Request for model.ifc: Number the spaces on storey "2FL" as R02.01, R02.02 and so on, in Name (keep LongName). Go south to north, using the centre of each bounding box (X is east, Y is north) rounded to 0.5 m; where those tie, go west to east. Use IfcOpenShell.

First a look at what the model holds.

```python
import ifcopenshell
import ifcopenshell.util.element
import ifcopenshell.util.placement

model = ifcopenshell.open("model.ifc")
print(model.schema)
storey = next(s for s in model.by_type("IfcBuildingStorey") if s.Name == "2FL")
spaces = [e for e in ifcopenshell.util.element.get_decomposition(storey) if e.is_a("IfcSpace")]
for e in sorted(spaces, key=lambda e: e.id()):
    origin = ifcopenshell.util.placement.get_local_placement(e.ObjectPlacement)[:3, 3]
    print(e.id(), e.Name, e.LongName, origin.round(2) + 0.0, sep=" | ")
```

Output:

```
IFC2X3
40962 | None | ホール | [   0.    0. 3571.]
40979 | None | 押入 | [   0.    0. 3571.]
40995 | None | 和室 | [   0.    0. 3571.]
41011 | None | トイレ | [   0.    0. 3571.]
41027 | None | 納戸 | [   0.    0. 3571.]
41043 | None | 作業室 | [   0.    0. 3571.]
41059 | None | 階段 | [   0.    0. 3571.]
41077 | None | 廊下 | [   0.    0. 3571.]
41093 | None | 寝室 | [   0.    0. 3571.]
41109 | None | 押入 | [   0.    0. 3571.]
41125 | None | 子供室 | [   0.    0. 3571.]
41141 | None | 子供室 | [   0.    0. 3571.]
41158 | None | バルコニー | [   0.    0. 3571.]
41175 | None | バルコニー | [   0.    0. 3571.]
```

```python
import ifcopenshell
import ifcopenshell.geom
import ifcopenshell.util.element
import ifcopenshell.util.shape

model = ifcopenshell.open("model.ifc")
settings = ifcopenshell.geom.settings()
settings.set("use-world-coords", True)


def centre(element):
    shape = ifcopenshell.geom.create_shape(settings, element)
    return ifcopenshell.util.shape.get_bbox_centroid(shape.geometry)


storey = next(s for s in model.by_type("IfcBuildingStorey") if s.Name == "2FL")
spaces = [e for e in ifcopenshell.util.element.get_decomposition(storey) if e.is_a("IfcSpace")]

# Insertion points can sit at a corner or the storey origin, so sort by the geometry (in metres).
centres = {e: centre(e) for e in spaces}
spaces.sort(key=lambda e: (round(centres[e][1] / 0.5), centres[e][0]))

for i, e in enumerate(spaces, start=1):
    number = f"R02.{i:02d}"
    e.Name = number
    print(e.id(), number)

model.write("model_updated.ifc")
```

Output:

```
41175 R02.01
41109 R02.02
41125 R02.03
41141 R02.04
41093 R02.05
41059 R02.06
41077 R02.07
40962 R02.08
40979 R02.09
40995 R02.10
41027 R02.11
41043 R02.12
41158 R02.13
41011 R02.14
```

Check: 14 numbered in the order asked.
